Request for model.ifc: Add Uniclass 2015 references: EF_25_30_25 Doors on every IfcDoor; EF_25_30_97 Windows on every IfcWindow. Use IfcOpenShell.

First a look at what the model holds.

```python
import ifcopenshell

model = ifcopenshell.open("model.ifc")
print(model.schema)
print("classifications:", [c.Name for c in model.by_type("IfcClassification")])
for ifc_class in ("IfcDoor", "IfcRoof", "IfcStair", "IfcWall", "IfcWindow"):
    print(ifc_class, len(model.by_type(ifc_class)))
```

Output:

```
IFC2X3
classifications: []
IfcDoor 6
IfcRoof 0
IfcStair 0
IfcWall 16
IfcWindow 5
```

```python
import ifcopenshell
import ifcopenshell.api.classification

model = ifcopenshell.open("model.ifc")

# IFC2X3 requires Source and Edition and has no link from the project to the system.
system = model.create_entity("IfcClassification", Source="NBS", Edition="2015", Name="Uniclass 2015")

codes = {
    "IfcDoor": ("EF_25_30_25", "Doors"),
    "IfcWindow": ("EF_25_30_97", "Windows"),
}
for ifc_class, (code, name) in codes.items():
    products = model.by_type(ifc_class)
    ifcopenshell.api.classification.add_reference(
        model, products=products, classification=system, identification=code, name=name
    )
    print(code, len(products))

model.write("model_v2.ifc")
```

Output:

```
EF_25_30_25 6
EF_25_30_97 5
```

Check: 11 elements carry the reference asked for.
